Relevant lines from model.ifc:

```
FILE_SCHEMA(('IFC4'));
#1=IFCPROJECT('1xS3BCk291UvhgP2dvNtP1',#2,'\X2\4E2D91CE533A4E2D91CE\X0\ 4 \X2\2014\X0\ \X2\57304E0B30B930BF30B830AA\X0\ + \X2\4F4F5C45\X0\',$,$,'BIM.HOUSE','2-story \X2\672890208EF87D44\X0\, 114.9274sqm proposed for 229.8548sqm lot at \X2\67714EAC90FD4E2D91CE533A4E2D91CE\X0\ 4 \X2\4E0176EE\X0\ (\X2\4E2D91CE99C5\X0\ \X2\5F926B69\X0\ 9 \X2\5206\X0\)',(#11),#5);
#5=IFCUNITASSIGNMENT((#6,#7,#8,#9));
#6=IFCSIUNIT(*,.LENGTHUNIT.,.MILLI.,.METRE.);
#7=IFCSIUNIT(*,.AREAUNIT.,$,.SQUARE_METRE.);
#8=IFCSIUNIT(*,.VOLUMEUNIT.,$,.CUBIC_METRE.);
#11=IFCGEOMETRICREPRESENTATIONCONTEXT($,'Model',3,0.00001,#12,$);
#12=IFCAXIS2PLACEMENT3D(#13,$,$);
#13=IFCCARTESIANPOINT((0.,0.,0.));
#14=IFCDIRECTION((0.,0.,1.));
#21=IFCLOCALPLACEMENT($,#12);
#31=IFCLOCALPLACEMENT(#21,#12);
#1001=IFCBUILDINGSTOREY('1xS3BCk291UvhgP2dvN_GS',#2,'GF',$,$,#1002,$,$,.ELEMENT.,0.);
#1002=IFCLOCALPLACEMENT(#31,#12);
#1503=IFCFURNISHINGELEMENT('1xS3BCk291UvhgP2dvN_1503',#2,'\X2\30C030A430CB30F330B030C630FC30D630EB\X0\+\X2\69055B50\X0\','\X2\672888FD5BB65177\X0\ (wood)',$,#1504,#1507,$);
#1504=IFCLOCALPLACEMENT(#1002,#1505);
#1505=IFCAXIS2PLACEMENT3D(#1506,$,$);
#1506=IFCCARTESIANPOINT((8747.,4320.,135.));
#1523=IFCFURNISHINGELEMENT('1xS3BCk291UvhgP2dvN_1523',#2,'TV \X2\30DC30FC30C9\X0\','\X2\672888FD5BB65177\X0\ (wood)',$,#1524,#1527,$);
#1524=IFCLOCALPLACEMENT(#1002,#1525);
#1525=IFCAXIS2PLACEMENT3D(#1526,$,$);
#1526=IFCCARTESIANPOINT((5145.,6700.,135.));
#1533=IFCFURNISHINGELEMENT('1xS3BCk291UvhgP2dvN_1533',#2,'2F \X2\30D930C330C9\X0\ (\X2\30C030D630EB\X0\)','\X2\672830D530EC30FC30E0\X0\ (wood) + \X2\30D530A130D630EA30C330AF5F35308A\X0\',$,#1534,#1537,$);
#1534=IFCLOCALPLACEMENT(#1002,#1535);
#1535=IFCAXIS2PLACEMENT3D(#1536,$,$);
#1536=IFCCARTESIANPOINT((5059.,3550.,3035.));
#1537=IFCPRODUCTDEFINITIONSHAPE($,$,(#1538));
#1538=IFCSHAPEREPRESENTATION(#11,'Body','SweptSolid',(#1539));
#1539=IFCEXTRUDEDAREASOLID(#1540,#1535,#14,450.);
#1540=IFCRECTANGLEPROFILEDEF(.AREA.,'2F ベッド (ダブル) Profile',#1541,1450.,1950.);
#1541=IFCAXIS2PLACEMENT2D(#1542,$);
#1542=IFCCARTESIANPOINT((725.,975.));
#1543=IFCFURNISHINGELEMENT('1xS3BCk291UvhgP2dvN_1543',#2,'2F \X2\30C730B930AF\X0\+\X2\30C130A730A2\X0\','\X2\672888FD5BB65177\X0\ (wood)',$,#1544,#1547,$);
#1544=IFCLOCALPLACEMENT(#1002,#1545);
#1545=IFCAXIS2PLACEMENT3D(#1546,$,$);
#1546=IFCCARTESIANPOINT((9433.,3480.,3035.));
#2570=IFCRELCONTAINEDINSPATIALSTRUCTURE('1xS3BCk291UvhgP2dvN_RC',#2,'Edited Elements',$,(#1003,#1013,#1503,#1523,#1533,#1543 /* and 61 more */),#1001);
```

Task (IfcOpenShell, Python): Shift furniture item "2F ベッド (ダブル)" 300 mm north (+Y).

```python
import ifcopenshell
import ifcopenshell.api.geometry
import ifcopenshell.util.placement
import ifcopenshell.util.unit

model = ifcopenshell.open("model.ifc")
unit_scale = ifcopenshell.util.unit.calculate_unit_scale(model)

item = model.by_guid("1xS3BCk291UvhgP2dvN_1533")
matrix = ifcopenshell.util.placement.get_local_placement(item.ObjectPlacement)
matrix[1, 3] += 0.3 / unit_scale
ifcopenshell.api.geometry.edit_object_placement(model, product=item, matrix=matrix, is_si=False)

print(ifcopenshell.util.placement.get_local_placement(item.ObjectPlacement).round(3) + 0.0)

model.write("model_updated.ifc")
```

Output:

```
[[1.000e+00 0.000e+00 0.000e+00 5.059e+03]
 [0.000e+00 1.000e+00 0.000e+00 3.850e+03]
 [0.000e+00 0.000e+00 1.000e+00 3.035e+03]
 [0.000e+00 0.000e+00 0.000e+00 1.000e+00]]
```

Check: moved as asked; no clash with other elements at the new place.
